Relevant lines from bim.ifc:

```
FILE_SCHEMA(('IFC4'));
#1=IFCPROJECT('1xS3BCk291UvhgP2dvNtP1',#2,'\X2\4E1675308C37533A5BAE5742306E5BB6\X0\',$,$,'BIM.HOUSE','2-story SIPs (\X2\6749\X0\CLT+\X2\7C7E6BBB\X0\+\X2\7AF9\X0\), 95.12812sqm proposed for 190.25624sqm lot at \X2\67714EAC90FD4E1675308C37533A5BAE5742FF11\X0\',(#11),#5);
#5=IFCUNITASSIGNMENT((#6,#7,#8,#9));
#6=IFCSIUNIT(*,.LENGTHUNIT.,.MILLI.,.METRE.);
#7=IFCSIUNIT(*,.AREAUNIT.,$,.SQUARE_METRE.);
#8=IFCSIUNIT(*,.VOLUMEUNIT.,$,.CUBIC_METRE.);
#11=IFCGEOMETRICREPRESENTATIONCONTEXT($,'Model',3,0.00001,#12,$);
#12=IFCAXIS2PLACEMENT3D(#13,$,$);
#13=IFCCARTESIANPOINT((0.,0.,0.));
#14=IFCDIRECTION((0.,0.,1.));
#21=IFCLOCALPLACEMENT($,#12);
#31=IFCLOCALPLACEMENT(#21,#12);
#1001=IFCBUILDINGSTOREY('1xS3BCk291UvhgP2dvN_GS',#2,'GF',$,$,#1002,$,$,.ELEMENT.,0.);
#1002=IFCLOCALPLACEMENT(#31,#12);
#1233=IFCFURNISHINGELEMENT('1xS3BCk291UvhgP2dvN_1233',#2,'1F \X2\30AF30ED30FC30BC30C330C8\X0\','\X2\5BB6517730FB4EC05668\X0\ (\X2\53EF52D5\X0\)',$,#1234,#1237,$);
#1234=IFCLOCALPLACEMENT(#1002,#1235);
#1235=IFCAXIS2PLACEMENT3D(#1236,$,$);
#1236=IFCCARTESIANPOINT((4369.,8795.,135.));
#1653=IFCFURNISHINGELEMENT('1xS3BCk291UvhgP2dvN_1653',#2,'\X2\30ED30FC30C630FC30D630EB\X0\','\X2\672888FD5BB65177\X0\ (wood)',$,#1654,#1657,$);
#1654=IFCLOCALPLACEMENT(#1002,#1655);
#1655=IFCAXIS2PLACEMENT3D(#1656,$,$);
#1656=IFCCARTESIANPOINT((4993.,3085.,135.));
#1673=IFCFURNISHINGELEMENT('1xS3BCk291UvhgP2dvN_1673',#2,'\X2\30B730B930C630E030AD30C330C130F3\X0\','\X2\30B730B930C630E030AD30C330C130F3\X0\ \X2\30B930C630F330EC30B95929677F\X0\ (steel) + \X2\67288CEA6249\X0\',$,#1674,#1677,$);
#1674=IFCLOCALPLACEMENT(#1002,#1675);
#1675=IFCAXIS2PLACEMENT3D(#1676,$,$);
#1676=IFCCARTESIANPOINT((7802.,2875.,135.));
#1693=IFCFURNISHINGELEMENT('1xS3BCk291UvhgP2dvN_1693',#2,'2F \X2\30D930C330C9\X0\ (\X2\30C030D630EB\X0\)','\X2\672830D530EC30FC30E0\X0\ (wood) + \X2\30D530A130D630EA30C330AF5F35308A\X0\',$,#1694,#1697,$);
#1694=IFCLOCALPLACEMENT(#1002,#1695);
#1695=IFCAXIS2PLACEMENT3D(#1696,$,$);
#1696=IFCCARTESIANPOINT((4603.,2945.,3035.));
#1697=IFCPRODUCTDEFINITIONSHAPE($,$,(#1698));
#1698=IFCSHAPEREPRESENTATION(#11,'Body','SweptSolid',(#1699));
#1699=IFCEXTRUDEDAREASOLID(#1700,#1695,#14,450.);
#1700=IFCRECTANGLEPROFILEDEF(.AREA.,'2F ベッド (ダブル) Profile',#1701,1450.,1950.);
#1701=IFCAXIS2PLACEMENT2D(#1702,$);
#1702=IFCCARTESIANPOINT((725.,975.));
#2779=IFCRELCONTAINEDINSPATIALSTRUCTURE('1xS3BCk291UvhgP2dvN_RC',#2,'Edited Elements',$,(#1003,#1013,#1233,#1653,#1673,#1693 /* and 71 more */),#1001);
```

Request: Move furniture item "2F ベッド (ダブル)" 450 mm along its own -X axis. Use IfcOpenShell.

```python
import ifcopenshell
import ifcopenshell.api.geometry
import ifcopenshell.util.placement
import ifcopenshell.util.unit

model = ifcopenshell.open("bim.ifc")
unit_scale = ifcopenshell.util.unit.calculate_unit_scale(model)

item = model.by_guid("1xS3BCk291UvhgP2dvN_1693")
matrix = ifcopenshell.util.placement.get_local_placement(item.ObjectPlacement)
matrix[:3, 3] -= matrix[:3, 0] * 0.45 / unit_scale
ifcopenshell.api.geometry.edit_object_placement(model, product=item, matrix=matrix, is_si=False)

print(ifcopenshell.util.placement.get_local_placement(item.ObjectPlacement).round(3) + 0.0)

model.write("bim_v2.ifc")
```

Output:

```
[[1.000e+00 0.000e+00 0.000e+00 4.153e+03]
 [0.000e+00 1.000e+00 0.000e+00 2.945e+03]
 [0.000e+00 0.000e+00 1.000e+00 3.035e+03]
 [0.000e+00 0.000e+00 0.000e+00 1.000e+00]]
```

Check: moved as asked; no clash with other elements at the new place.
